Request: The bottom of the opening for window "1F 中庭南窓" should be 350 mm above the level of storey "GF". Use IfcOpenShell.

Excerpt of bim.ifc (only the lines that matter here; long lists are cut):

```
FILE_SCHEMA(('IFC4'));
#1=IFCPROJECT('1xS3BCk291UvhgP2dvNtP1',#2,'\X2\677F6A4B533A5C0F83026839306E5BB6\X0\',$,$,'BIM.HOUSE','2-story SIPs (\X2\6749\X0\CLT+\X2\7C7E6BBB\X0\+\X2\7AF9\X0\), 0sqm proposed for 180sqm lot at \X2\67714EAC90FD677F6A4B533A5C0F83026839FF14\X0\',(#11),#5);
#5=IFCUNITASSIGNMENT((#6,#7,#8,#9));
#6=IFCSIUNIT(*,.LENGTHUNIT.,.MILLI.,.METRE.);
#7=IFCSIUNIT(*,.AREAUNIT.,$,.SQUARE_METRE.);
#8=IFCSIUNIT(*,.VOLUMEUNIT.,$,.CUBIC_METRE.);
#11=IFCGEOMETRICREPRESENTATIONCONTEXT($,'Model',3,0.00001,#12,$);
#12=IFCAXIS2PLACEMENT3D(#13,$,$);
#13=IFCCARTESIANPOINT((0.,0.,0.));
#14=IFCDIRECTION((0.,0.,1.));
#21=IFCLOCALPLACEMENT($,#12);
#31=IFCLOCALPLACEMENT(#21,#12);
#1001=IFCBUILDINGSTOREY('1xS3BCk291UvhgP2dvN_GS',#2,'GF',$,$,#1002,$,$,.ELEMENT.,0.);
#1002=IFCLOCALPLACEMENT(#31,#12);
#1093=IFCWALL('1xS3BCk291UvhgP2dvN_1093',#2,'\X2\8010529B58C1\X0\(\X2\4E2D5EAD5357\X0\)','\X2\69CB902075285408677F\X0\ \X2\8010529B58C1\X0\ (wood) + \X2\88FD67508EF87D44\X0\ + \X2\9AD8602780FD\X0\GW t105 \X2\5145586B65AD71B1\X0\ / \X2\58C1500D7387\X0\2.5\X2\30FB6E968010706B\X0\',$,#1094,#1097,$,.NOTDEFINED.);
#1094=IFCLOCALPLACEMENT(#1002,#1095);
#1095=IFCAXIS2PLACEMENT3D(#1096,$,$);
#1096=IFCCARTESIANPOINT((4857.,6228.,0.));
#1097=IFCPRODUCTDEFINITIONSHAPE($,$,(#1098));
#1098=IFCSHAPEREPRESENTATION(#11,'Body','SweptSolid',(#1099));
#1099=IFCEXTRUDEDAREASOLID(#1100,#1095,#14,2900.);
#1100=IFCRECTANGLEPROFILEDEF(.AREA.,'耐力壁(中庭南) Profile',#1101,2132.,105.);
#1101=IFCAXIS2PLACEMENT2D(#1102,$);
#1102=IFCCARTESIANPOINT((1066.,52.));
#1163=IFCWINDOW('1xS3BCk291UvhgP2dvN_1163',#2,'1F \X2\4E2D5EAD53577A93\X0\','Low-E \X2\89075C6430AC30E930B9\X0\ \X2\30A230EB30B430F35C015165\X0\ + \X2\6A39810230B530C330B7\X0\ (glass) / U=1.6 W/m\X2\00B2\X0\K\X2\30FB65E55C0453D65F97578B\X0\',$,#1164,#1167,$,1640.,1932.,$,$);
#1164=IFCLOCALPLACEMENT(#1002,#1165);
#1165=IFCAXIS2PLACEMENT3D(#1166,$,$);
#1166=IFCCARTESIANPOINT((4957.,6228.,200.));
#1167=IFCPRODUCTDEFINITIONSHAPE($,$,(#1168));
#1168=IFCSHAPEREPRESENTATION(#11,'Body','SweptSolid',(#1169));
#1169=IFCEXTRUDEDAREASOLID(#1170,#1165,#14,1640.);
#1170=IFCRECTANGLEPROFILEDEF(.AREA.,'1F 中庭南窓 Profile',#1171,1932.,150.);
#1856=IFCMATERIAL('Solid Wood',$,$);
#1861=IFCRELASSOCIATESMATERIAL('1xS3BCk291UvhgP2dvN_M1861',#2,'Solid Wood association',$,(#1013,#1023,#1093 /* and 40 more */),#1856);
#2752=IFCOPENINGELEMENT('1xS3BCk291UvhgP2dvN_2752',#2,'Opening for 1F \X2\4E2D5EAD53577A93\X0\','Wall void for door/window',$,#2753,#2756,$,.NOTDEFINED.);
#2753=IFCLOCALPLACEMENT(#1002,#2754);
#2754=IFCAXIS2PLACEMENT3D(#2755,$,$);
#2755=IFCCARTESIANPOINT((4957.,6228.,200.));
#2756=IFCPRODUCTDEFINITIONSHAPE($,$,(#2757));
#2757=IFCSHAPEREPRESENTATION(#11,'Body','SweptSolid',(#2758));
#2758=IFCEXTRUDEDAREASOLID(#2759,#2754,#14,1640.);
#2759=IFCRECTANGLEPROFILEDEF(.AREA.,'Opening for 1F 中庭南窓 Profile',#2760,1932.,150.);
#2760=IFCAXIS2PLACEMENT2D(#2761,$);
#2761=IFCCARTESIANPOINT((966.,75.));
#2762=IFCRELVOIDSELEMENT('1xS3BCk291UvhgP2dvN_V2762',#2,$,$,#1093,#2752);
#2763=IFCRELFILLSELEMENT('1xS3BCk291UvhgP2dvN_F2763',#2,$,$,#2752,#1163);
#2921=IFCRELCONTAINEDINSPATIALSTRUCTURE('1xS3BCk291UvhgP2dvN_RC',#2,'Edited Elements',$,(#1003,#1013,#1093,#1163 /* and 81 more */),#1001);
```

```python
import numpy as np
import ifcopenshell
import ifcopenshell.api.geometry
import ifcopenshell.geom
import ifcopenshell.util.element
import ifcopenshell.util.placement
import ifcopenshell.util.shape
import ifcopenshell.util.unit

model = ifcopenshell.open("bim.ifc")
unit_scale = ifcopenshell.util.unit.calculate_unit_scale(model)

window = model.by_id(1163)
opening = window.FillsVoids[0].RelatingOpeningElement
storey = ifcopenshell.util.element.get_container(window, ifc_class="IfcBuildingStorey")
level = ifcopenshell.util.placement.get_local_placement(storey.ObjectPlacement)[2, 3]

# The opening's origin need not be at the sill, so measure its lowest point.
shape = ifcopenshell.geom.create_shape(ifcopenshell.geom.settings(), opening)
bottom = ifcopenshell.util.shape.get_shape_bottom_elevation(shape, shape.geometry) / unit_scale
dz = level + 0.35 / unit_scale - bottom

shift = np.array([0.0, 0.0, dz])
# The window is not placed relative to its opening, so move both.
for product in (opening, window):
    matrix = ifcopenshell.util.placement.get_local_placement(product.ObjectPlacement)
    matrix[:3, 3] += shift
    ifcopenshell.api.geometry.edit_object_placement(model, product=product, matrix=matrix, is_si=False)

print(f"moved by {dz * unit_scale:+.3f} m")

model.write("bim_edited.ifc")
```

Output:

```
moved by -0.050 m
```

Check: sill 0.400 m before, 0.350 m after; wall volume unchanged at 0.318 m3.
